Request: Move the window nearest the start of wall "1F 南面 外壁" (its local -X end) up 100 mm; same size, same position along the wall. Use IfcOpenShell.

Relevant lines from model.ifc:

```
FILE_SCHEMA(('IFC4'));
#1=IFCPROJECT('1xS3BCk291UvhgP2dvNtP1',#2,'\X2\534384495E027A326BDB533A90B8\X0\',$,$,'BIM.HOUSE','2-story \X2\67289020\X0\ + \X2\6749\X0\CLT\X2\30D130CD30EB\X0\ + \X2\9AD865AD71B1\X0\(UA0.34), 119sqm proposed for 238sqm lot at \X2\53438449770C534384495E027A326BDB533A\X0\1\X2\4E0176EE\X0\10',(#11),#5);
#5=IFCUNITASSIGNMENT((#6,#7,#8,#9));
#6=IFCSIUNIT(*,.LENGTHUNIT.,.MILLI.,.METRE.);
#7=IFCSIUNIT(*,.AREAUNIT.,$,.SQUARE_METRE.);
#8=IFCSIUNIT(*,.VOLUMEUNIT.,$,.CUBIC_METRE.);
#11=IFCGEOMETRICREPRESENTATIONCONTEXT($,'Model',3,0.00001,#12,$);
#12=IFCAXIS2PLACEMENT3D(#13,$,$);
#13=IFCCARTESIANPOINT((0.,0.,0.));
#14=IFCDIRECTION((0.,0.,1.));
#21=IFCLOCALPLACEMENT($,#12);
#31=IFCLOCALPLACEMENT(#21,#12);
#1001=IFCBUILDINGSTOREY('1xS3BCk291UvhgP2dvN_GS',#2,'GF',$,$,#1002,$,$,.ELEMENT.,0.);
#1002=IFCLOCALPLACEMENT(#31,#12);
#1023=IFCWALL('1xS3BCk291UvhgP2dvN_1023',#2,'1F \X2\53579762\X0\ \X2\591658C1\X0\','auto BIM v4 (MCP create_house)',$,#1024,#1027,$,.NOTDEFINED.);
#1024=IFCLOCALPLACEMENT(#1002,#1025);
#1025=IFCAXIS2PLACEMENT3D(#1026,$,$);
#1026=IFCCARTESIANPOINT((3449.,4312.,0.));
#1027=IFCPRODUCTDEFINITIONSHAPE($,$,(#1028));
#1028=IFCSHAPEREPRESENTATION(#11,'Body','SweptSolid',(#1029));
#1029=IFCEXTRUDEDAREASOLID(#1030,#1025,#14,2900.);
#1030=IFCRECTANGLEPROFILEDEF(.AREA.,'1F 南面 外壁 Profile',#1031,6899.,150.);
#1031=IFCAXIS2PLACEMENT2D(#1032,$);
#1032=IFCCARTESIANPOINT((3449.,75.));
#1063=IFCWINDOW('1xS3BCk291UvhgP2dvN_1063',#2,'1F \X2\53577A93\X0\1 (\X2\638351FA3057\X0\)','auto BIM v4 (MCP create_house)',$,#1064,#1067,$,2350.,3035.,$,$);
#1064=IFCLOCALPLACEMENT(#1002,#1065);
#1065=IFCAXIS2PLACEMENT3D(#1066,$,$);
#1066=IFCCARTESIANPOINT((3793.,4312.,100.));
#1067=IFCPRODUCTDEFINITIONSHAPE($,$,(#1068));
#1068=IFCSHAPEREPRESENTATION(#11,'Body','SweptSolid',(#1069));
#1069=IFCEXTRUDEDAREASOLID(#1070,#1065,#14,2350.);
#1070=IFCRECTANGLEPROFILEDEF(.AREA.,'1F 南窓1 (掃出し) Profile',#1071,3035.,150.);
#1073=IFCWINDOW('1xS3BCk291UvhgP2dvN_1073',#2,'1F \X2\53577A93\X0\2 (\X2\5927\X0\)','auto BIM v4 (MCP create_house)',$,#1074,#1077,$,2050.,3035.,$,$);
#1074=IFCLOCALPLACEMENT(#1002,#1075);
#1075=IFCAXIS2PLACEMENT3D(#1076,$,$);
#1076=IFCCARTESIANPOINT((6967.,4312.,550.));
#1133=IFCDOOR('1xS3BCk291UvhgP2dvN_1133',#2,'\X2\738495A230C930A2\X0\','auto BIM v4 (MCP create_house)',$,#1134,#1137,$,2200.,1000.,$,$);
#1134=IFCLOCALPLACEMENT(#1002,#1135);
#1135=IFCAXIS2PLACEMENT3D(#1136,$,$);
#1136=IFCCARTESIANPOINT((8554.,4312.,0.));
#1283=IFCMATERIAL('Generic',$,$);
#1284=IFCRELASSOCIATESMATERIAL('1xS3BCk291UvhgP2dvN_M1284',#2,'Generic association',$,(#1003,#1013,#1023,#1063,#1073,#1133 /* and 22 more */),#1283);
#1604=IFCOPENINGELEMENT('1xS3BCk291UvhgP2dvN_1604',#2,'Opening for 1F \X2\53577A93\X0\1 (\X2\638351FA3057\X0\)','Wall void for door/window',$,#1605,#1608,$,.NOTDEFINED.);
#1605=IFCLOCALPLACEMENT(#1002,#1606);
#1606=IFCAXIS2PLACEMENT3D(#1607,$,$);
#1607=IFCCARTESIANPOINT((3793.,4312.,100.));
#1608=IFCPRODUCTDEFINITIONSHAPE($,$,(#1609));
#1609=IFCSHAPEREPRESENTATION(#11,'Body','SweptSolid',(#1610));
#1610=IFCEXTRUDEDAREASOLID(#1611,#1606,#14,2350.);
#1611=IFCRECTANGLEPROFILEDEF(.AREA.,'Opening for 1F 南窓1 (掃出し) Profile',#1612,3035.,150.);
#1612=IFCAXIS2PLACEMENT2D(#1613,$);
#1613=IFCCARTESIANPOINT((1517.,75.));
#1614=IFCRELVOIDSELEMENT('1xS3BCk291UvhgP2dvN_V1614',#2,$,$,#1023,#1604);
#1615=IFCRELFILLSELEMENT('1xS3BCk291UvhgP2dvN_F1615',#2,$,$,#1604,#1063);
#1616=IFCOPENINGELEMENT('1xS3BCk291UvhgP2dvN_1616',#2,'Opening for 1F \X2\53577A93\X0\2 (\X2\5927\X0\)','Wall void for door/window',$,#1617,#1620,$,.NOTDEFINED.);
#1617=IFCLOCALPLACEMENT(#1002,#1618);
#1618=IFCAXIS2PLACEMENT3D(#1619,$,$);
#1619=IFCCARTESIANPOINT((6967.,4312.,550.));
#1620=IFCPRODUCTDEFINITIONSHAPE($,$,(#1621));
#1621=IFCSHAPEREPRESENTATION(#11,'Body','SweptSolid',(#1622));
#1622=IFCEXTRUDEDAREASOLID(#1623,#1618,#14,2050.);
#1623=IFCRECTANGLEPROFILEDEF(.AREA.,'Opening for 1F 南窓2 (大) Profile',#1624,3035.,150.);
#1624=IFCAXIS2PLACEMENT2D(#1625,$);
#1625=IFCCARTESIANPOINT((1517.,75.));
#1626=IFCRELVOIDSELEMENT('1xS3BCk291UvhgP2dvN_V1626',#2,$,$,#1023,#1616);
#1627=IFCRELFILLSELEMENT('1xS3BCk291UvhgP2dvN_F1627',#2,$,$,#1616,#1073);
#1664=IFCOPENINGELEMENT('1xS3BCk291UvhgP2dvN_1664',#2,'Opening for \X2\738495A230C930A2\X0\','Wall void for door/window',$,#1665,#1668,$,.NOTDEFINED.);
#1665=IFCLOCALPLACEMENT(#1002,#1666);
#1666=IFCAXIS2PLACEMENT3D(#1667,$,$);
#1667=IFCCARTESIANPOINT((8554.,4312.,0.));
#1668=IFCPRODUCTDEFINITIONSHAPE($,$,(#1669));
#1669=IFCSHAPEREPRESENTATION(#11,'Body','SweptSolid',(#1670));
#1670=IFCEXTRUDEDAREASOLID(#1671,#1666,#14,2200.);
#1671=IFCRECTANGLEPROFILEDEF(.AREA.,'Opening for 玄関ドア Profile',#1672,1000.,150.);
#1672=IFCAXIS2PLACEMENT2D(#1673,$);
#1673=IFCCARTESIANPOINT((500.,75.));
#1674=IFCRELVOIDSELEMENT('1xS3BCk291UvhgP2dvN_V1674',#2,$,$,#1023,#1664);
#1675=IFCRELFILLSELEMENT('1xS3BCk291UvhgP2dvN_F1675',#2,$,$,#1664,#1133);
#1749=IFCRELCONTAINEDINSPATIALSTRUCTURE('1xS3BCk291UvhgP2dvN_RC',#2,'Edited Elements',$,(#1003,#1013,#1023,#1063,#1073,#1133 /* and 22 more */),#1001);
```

```python
import numpy as np
import ifcopenshell
import ifcopenshell.api.geometry
import ifcopenshell.util.placement
import ifcopenshell.util.unit

model = ifcopenshell.open("model.ifc")
unit_scale = ifcopenshell.util.unit.calculate_unit_scale(model)

window = model.by_guid("1xS3BCk291UvhgP2dvN_1063")
opening = window.FillsVoids[0].RelatingOpeningElement
dz = 100.0

shift = np.array([0.0, 0.0, dz])
# The window is not placed relative to its opening, so move both.
for product in (opening, window):
    matrix = ifcopenshell.util.placement.get_local_placement(product.ObjectPlacement)
    matrix[:3, 3] += shift
    ifcopenshell.api.geometry.edit_object_placement(model, product=product, matrix=matrix, is_si=False)

print(f"moved by {dz * unit_scale:+.3f} m")

model.write("model_updated.ifc")
```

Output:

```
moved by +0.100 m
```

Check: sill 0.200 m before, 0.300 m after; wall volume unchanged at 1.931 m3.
